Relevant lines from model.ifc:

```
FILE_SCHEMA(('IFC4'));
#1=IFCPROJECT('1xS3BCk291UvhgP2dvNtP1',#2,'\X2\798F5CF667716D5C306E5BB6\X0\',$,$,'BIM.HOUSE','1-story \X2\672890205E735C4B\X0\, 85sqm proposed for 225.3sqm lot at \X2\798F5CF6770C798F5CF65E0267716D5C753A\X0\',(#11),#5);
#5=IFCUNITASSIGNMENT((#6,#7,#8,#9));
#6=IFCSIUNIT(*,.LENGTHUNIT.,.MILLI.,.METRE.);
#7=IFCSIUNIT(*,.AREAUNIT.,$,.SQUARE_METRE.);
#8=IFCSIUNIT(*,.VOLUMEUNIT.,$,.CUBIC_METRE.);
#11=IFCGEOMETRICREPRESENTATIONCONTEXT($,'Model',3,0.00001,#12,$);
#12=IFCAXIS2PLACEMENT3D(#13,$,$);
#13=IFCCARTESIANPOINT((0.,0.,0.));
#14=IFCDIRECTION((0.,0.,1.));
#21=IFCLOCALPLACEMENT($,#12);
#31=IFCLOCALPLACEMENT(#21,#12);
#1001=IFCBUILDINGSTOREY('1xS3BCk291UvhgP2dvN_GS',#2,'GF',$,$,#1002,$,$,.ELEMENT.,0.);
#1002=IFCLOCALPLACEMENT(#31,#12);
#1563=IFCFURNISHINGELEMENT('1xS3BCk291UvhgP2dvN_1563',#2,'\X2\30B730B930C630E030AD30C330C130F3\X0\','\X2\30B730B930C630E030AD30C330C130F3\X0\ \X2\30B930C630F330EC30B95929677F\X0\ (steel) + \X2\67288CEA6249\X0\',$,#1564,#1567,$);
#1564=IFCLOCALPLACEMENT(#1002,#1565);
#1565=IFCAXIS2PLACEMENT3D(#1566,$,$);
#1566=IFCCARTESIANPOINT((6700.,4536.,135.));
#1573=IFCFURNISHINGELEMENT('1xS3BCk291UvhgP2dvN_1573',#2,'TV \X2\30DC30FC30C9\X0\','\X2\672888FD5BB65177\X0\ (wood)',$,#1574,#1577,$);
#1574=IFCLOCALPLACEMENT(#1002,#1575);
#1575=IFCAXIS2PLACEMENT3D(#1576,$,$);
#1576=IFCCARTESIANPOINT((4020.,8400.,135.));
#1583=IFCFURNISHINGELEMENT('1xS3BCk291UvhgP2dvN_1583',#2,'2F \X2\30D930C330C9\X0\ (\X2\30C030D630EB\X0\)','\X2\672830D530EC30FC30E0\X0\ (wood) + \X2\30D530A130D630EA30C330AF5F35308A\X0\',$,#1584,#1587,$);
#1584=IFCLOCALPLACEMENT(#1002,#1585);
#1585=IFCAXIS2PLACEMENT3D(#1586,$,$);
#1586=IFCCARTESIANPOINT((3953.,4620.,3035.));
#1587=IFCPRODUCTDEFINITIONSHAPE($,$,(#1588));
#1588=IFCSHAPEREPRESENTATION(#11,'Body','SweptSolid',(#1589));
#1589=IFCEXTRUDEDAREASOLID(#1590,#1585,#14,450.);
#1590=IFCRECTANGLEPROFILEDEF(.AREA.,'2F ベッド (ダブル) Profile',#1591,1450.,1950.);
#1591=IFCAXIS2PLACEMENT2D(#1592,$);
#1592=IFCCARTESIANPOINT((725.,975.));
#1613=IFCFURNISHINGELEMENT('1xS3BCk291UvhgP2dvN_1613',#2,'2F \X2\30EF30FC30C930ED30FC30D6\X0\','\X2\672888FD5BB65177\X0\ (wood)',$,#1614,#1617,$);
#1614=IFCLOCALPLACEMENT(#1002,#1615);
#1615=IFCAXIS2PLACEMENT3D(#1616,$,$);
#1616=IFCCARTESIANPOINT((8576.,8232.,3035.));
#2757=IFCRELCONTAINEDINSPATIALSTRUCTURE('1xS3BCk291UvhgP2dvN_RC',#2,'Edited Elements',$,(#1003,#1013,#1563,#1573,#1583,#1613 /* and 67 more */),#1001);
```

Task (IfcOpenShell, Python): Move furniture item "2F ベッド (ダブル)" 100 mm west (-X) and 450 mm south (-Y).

```python
import ifcopenshell
import ifcopenshell.api.geometry
import ifcopenshell.util.placement
import ifcopenshell.util.unit

model = ifcopenshell.open("model.ifc")
unit_scale = ifcopenshell.util.unit.calculate_unit_scale(model)

item = model.by_guid("1xS3BCk291UvhgP2dvN_1583")
matrix = ifcopenshell.util.placement.get_local_placement(item.ObjectPlacement)
matrix[0, 3] -= 0.1 / unit_scale
matrix[1, 3] -= 0.45 / unit_scale
ifcopenshell.api.geometry.edit_object_placement(model, product=item, matrix=matrix, is_si=False)

print(ifcopenshell.util.placement.get_local_placement(item.ObjectPlacement).round(3) + 0.0)

model.write("model_updated.ifc")
```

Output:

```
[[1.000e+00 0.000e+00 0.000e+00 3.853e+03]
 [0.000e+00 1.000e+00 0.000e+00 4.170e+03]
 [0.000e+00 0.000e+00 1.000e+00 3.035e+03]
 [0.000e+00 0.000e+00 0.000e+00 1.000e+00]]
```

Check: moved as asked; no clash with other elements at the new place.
